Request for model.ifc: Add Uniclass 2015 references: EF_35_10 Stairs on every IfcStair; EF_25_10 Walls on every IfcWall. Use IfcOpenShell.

First a look at what the model holds.

```python
import ifcopenshell

model = ifcopenshell.open("model.ifc")
print(model.schema)
print("classifications:", [c.Name for c in model.by_type("IfcClassification")])
for ifc_class in ("IfcDoor", "IfcRoof", "IfcStair", "IfcWall", "IfcWindow"):
    print(ifc_class, len(model.by_type(ifc_class)))
```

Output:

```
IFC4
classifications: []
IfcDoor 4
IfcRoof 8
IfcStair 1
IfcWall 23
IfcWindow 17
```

```python
import ifcopenshell
import ifcopenshell.api.classification

model = ifcopenshell.open("model.ifc")

system = ifcopenshell.api.classification.add_classification(model, classification="Uniclass 2015")

codes = {
    "IfcStair": ("EF_35_10", "Stairs"),
    "IfcWall": ("EF_25_10", "Walls"),
}
for ifc_class, (code, name) in codes.items():
    products = model.by_type(ifc_class)
    ifcopenshell.api.classification.add_reference(
        model, products=products, classification=system, identification=code, name=name
    )
    print(code, len(products))

model.write("model_edited.ifc")
```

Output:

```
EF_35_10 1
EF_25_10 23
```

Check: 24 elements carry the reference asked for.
